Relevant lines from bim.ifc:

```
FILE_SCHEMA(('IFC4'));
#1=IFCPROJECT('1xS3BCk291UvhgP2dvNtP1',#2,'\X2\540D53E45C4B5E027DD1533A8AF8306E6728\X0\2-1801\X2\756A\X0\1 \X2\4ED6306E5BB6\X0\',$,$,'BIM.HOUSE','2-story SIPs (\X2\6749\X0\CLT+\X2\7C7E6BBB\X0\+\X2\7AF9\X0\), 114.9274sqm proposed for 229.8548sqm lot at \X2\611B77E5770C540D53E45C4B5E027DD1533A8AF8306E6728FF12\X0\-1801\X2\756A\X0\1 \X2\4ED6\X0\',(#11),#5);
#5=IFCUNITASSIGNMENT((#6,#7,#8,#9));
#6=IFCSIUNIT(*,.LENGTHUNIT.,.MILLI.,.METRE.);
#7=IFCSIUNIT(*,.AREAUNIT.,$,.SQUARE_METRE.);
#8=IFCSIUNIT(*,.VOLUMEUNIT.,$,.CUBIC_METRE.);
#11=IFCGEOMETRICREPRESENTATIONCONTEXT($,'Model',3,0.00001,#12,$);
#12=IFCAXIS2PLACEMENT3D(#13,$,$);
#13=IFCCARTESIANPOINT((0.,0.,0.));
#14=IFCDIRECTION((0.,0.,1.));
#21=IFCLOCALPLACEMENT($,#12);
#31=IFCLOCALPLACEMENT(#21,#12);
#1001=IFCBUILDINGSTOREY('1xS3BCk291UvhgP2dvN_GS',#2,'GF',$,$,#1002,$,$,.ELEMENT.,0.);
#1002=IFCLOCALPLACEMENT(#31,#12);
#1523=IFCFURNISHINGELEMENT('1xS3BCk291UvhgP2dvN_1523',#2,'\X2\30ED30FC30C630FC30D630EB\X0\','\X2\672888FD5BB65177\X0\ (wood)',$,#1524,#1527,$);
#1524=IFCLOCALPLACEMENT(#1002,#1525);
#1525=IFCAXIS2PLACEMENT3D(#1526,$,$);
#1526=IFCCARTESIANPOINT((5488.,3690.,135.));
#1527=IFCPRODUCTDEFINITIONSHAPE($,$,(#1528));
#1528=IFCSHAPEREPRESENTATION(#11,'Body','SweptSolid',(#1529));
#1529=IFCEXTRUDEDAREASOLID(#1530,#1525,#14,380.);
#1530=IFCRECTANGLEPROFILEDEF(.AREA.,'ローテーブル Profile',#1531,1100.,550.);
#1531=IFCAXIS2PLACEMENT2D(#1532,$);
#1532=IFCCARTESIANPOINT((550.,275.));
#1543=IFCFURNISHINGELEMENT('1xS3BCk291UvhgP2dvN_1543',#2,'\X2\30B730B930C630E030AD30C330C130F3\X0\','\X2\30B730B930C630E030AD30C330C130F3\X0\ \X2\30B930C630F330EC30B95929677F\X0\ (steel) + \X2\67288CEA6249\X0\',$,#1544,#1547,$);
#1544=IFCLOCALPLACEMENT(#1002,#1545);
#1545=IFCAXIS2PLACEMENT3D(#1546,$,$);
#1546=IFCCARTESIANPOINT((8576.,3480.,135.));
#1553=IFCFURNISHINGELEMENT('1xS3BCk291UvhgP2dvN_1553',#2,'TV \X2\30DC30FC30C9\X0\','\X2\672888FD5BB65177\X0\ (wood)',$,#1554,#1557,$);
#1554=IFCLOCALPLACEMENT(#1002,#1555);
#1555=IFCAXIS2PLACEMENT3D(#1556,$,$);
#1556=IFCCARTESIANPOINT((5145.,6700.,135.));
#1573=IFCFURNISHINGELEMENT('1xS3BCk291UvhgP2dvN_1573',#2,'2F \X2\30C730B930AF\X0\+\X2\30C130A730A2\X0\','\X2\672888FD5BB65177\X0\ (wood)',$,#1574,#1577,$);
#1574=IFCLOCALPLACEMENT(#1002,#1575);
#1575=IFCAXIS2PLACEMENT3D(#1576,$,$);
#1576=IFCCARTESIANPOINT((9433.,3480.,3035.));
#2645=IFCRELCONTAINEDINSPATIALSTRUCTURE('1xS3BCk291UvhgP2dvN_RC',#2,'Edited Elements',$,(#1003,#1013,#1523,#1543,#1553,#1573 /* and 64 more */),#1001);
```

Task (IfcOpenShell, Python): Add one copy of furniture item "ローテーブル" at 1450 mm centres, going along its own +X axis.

```python
import ifcopenshell
import ifcopenshell.api.geometry
import ifcopenshell.api.root
import ifcopenshell.util.element
import ifcopenshell.util.placement

model = ifcopenshell.open("bim.ifc")


def reuse_history(source, copy):
    """copy_class also copies each property set's owner history, people and application; keep the originals."""
    for rel in copy.IsDefinedBy:
        if rel.is_a("IfcRelDefinesByProperties") and (history := rel.RelatingPropertyDefinition.OwnerHistory):
            rel.RelatingPropertyDefinition.OwnerHistory = source.OwnerHistory
            ifcopenshell.util.element.remove_deep2(model, history)


source = model.by_id(1523)
base = ifcopenshell.util.placement.get_local_placement(source.ObjectPlacement)
step = base[:3, 0] * 1450.0

for i in range(1, 2):
    copy = ifcopenshell.api.root.copy_class(model, product=source)
    copy.Representation = ifcopenshell.util.element.copy_deep(
        model, source.Representation, exclude=["IfcGeometricRepresentationContext", "IfcRepresentationMap"]
    )
    reuse_history(source, copy)
    matrix = base.copy()
    matrix[:3, 3] += i * step
    print("added at", matrix[:3, 3].round(3) + 0.0)
    ifcopenshell.api.geometry.edit_object_placement(model, product=copy, matrix=matrix, is_si=False)

model.write("bim_edited.ifc")
```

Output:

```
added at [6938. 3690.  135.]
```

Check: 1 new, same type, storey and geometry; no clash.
